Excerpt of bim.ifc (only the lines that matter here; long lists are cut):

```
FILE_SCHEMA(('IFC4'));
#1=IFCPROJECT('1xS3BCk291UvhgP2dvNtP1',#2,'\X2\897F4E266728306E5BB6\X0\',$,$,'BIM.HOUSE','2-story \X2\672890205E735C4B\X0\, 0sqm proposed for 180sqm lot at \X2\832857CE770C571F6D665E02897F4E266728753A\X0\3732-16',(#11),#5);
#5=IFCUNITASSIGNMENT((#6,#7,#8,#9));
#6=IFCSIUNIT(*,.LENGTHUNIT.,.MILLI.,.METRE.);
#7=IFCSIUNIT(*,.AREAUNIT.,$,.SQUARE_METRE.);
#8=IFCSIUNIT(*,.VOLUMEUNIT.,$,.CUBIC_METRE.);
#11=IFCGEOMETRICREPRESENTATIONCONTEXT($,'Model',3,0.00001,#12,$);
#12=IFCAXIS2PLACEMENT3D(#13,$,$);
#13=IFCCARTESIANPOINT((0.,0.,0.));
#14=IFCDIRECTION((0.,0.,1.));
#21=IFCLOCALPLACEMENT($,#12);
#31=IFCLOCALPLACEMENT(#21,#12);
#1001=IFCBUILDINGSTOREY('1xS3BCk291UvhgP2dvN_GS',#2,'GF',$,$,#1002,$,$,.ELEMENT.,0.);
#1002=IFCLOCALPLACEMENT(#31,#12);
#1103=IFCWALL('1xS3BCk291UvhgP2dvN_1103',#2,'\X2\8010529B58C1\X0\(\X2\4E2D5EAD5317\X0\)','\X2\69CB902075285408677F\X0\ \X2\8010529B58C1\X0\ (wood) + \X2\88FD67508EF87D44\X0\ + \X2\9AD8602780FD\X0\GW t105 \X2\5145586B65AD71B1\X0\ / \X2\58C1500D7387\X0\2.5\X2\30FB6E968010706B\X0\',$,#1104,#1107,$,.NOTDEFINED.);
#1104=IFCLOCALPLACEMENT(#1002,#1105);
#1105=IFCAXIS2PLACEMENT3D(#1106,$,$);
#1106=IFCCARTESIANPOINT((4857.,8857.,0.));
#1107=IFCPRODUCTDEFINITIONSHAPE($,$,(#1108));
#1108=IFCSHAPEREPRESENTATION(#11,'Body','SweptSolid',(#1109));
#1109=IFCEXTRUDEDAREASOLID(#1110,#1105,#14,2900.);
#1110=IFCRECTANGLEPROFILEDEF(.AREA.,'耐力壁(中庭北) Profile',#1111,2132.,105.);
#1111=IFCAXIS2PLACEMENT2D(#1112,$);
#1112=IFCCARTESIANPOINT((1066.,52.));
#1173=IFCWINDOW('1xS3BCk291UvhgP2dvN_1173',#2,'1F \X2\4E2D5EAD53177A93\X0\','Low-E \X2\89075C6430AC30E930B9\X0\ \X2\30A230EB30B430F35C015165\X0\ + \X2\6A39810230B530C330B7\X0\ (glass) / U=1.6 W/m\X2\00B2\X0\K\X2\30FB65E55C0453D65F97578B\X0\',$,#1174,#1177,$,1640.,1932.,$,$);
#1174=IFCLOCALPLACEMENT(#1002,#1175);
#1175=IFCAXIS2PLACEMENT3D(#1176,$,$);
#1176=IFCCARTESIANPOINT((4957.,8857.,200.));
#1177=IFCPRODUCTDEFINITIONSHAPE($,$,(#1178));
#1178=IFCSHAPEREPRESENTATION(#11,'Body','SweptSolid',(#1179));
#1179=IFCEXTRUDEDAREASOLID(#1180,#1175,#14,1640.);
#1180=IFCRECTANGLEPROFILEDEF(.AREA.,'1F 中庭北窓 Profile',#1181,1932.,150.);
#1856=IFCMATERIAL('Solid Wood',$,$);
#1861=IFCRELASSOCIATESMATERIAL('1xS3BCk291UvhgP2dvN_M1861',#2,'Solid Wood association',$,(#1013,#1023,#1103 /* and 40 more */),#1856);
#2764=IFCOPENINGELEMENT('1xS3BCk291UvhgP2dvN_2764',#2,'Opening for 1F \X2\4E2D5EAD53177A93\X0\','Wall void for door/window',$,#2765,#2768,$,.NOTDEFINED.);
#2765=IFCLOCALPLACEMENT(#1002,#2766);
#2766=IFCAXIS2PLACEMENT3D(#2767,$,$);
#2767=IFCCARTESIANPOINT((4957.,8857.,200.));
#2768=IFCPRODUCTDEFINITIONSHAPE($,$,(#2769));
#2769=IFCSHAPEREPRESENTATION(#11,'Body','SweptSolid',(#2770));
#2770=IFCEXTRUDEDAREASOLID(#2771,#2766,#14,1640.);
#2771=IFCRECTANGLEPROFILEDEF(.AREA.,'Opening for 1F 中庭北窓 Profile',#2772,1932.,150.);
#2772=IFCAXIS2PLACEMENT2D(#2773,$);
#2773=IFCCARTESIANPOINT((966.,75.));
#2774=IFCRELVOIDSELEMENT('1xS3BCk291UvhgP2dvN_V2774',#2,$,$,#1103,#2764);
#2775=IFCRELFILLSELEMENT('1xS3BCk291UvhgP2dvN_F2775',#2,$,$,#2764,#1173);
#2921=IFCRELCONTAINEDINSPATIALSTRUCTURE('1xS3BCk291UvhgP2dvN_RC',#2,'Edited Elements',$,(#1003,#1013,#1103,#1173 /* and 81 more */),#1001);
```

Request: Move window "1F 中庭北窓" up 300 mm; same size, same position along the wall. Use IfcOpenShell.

```python
import numpy as np
import ifcopenshell
import ifcopenshell.api.geometry
import ifcopenshell.util.placement
import ifcopenshell.util.unit

model = ifcopenshell.open("bim.ifc")
unit_scale = ifcopenshell.util.unit.calculate_unit_scale(model)

window = model.by_guid("1xS3BCk291UvhgP2dvN_1173")
opening = window.FillsVoids[0].RelatingOpeningElement
dz = 300.0

shift = np.array([0.0, 0.0, dz])
# The window is not placed relative to its opening, so move both.
for product in (opening, window):
    matrix = ifcopenshell.util.placement.get_local_placement(product.ObjectPlacement)
    matrix[:3, 3] += shift
    ifcopenshell.api.geometry.edit_object_placement(model, product=product, matrix=matrix, is_si=False)

print(f"moved by {dz * unit_scale:+.3f} m")

model.write("bim-out.ifc")
```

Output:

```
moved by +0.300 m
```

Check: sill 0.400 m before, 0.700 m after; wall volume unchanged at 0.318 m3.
